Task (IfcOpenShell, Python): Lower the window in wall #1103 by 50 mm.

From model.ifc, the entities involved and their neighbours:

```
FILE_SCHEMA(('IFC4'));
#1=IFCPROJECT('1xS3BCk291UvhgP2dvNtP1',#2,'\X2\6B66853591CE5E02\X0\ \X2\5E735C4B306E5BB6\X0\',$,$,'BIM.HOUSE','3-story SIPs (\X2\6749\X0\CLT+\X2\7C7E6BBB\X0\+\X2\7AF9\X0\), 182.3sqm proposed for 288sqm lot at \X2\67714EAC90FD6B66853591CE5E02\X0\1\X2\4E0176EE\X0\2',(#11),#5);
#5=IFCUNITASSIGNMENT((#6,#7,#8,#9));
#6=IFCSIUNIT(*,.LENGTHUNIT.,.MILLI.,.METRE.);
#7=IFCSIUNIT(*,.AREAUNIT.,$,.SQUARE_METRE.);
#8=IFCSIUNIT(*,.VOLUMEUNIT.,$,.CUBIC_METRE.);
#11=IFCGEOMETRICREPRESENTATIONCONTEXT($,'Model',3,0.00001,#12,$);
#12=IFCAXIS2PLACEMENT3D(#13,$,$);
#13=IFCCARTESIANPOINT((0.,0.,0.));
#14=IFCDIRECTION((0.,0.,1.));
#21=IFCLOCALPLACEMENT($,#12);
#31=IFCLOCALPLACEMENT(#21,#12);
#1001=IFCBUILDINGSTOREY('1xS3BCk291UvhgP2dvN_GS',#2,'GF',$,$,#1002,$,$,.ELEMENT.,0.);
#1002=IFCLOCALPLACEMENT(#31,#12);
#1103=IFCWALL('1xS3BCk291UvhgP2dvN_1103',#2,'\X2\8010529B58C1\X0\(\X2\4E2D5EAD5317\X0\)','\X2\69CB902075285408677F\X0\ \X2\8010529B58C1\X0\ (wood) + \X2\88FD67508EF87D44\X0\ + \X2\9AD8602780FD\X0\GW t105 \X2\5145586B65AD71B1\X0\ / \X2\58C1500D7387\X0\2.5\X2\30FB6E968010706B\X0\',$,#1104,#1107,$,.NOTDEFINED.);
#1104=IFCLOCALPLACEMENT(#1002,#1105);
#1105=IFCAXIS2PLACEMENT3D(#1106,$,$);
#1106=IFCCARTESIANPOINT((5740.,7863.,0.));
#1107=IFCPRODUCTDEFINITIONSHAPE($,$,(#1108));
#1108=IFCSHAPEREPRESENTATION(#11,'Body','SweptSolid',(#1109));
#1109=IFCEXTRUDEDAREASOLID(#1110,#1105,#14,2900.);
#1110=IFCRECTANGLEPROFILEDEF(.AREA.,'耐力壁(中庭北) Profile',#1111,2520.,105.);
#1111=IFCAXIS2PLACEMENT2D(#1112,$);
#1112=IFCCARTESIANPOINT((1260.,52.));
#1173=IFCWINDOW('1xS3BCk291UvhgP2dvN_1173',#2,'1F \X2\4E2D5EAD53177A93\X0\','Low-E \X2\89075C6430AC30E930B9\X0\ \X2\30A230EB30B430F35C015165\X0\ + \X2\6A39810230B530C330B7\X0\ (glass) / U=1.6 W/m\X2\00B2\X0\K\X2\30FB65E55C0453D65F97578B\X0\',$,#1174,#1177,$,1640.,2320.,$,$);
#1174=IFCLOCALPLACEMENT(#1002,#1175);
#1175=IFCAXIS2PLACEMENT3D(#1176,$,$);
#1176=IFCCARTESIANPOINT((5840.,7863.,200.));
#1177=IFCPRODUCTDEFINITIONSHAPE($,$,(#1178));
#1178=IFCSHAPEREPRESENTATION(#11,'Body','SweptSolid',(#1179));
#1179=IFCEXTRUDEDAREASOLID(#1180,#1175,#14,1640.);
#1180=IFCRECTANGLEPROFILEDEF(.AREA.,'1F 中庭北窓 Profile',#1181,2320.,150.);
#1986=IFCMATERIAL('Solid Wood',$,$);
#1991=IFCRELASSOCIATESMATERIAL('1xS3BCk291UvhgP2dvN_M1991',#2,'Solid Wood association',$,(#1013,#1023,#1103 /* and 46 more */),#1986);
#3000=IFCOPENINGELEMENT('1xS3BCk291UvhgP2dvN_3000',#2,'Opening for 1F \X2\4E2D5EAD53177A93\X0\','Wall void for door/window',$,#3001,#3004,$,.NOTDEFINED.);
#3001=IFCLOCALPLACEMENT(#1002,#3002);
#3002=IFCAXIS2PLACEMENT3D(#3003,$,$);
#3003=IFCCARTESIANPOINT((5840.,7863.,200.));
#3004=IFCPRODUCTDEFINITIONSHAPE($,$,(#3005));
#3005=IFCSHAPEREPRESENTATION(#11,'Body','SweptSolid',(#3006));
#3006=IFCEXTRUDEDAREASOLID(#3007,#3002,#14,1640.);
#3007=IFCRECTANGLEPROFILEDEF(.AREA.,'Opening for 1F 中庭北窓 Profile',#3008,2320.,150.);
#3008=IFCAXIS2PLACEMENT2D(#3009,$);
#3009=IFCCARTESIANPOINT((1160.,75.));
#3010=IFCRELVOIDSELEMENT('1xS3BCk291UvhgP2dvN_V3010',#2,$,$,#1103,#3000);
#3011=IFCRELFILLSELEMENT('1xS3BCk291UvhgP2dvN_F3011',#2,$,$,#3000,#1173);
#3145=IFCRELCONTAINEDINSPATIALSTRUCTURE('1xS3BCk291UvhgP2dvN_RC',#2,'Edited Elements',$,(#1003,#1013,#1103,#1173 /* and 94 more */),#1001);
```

```python
import numpy as np
import ifcopenshell
import ifcopenshell.api.geometry
import ifcopenshell.util.placement
import ifcopenshell.util.unit

model = ifcopenshell.open("model.ifc")
unit_scale = ifcopenshell.util.unit.calculate_unit_scale(model)

window = model.by_id(1173)
opening = window.FillsVoids[0].RelatingOpeningElement
dz = -50.0

shift = np.array([0.0, 0.0, dz])
# The window is not placed relative to its opening, so move both.
for product in (opening, window):
    matrix = ifcopenshell.util.placement.get_local_placement(product.ObjectPlacement)
    matrix[:3, 3] += shift
    ifcopenshell.api.geometry.edit_object_placement(model, product=product, matrix=matrix, is_si=False)

print(f"moved by {dz * unit_scale:+.3f} m")

model.write("model-out.ifc")
```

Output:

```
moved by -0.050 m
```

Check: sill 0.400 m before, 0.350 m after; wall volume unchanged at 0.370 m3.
